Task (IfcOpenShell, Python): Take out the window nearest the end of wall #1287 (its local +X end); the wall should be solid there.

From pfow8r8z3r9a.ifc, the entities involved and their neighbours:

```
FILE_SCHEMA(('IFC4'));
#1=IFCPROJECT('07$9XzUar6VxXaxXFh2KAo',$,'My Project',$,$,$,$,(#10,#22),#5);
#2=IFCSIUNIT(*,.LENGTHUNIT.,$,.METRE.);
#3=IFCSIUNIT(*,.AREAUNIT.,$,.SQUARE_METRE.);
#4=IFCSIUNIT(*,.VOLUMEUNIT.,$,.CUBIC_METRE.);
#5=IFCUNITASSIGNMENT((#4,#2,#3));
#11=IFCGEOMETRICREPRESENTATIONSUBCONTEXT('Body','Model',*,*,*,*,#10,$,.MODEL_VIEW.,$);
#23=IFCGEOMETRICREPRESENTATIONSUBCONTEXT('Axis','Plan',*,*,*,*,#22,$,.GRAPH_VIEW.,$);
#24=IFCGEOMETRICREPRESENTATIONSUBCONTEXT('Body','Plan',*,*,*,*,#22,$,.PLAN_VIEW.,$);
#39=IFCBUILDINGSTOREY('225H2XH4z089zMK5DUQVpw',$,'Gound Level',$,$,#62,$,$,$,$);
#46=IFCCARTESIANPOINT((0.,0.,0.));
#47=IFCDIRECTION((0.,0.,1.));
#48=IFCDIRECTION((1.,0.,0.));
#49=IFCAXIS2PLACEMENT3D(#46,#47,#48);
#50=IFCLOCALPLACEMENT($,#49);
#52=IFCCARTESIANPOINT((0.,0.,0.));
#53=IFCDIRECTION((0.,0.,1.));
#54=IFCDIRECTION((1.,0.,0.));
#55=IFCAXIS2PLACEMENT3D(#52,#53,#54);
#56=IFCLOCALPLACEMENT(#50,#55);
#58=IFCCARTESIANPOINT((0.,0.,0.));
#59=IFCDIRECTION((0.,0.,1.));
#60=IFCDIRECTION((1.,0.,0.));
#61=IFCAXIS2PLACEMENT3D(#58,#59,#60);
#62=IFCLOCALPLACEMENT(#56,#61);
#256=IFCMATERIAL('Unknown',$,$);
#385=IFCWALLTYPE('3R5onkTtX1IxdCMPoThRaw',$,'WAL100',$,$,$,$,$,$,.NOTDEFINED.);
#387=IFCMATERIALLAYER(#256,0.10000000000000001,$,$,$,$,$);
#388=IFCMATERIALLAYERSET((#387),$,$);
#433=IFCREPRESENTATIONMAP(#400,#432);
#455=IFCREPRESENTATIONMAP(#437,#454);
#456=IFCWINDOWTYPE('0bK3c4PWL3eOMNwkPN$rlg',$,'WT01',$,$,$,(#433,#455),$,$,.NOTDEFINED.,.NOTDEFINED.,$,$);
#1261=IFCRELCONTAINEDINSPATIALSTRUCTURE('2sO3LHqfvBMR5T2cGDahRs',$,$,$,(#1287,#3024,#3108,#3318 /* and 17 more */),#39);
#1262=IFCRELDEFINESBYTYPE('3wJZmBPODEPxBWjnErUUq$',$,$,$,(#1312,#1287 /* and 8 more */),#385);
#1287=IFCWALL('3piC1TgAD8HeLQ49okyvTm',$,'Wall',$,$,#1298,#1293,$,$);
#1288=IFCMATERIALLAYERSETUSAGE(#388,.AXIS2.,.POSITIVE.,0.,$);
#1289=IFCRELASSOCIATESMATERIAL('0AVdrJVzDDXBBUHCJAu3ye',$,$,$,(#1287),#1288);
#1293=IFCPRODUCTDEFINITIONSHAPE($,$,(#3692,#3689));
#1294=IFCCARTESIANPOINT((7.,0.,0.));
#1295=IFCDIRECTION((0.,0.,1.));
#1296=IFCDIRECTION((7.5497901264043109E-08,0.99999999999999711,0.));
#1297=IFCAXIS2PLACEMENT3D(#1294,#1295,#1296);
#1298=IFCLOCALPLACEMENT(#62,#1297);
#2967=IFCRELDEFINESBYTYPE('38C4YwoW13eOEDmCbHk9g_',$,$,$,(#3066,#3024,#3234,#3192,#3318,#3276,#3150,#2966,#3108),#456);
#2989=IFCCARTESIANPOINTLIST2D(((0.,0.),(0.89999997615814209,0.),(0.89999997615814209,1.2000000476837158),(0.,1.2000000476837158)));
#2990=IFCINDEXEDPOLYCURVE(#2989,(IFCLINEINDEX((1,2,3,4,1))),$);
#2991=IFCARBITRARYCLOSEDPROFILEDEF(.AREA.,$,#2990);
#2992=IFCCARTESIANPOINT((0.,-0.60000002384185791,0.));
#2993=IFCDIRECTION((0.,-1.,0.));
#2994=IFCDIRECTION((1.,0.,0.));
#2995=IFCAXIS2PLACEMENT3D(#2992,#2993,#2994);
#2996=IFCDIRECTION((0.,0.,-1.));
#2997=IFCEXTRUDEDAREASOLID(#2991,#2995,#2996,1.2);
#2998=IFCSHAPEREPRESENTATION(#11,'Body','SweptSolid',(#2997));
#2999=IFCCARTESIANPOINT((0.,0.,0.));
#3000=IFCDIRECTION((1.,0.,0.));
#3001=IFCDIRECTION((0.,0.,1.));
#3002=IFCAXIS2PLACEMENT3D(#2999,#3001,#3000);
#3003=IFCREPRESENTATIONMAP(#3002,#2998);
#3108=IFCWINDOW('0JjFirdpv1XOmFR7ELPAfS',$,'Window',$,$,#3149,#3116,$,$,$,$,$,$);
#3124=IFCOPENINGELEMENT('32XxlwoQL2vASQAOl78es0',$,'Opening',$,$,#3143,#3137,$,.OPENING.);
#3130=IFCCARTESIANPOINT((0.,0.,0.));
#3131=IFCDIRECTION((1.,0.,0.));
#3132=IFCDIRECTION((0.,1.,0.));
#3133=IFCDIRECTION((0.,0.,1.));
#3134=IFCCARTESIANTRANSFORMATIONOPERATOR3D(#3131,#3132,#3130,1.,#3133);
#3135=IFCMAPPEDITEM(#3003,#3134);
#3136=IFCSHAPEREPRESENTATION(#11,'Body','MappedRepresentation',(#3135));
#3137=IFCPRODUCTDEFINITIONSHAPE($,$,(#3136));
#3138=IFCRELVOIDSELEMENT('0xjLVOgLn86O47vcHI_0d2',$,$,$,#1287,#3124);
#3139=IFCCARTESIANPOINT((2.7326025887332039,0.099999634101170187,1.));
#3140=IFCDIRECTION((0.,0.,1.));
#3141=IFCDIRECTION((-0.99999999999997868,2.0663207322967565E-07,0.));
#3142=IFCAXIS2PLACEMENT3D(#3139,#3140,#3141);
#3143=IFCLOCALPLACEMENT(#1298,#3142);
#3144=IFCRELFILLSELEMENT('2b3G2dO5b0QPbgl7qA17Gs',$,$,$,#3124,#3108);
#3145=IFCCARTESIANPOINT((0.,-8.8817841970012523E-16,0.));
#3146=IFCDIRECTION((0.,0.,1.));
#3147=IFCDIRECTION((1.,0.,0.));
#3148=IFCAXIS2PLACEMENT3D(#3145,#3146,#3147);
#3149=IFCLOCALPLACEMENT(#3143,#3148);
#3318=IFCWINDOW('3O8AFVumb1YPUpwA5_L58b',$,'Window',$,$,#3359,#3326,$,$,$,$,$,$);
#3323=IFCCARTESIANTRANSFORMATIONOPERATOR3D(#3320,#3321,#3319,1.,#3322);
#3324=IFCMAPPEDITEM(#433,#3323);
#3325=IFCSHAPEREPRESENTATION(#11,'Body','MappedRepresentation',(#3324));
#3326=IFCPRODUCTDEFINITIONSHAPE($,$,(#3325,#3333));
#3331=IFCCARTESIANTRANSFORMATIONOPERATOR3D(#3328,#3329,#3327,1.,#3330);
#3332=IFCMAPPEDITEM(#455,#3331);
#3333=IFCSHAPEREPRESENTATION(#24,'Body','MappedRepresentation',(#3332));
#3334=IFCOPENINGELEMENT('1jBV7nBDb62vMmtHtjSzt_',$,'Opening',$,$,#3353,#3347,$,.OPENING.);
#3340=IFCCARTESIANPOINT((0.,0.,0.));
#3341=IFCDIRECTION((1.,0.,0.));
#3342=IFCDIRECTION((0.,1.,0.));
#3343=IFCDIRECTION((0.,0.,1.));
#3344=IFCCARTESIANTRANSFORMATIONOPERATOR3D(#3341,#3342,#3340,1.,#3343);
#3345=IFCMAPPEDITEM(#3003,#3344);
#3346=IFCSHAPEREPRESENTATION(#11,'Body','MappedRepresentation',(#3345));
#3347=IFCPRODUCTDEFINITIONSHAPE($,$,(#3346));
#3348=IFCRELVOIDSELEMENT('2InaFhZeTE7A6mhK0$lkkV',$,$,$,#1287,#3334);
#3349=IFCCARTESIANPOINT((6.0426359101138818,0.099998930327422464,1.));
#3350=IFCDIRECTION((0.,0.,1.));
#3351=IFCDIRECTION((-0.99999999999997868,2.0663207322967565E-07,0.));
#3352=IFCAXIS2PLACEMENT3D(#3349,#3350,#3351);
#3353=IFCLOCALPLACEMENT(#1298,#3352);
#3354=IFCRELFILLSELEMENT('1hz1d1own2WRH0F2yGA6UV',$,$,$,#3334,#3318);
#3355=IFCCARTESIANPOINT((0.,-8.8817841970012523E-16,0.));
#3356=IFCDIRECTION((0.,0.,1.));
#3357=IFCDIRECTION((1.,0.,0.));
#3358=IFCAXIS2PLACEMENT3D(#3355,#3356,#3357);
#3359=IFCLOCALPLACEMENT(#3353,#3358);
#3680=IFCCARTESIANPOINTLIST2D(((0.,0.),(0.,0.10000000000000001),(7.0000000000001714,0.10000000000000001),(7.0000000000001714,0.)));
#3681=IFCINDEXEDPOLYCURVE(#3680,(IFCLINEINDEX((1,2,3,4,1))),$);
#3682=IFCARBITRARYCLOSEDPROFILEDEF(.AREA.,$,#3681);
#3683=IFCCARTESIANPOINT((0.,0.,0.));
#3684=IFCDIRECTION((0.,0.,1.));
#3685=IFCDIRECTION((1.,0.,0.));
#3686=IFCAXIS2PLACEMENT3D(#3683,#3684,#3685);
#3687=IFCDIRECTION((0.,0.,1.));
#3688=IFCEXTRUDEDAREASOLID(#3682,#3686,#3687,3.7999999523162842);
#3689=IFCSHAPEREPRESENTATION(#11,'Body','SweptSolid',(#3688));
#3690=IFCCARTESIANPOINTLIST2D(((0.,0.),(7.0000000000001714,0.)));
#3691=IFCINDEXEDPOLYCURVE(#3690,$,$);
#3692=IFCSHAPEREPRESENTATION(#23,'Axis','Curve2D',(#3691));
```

```python
import ifcopenshell
import ifcopenshell.api.feature
import ifcopenshell.api.root
import ifcopenshell.geom
import ifcopenshell.util.shape

model = ifcopenshell.open("pfow8r8z3r9a.ifc")
settings = ifcopenshell.geom.settings()


def volume(element):
    """Net volume in cubic metres, openings subtracted."""
    shape = ifcopenshell.geom.create_shape(settings, element)
    return ifcopenshell.util.shape.get_volume(shape.geometry)


window = model.by_guid("3O8AFVumb1YPUpwA5_L58b")
opening = window.FillsVoids[0].RelatingOpeningElement
wall = opening.VoidsElements[0].RelatingBuildingElement
before = volume(wall)

ifcopenshell.api.root.remove_product(model, product=window)
ifcopenshell.api.feature.remove_feature(model, feature=opening)

after = volume(wall)

print(f"wall volume {before:.3f} -> {after:.3f} m3")

model.write("pfow8r8z3r9a-out.ifc")
```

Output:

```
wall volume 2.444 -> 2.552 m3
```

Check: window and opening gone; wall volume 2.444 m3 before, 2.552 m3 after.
